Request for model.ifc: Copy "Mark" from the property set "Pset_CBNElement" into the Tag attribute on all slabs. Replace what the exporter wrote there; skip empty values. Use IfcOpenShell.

First a look at what the model holds.

```python
import ifcopenshell
import ifcopenshell.util.element

model = ifcopenshell.open("model.ifc")
print(model.schema)
slabs = model.by_type("IfcSlab")
print(len(slabs), "slabs")
for e in slabs[:8]:
    source = ifcopenshell.util.element.get_pset(e, "Pset_CBNElement", "Mark")
    target = e.Tag
    print(e.id(), repr(source), repr(target), sep=" | ")
```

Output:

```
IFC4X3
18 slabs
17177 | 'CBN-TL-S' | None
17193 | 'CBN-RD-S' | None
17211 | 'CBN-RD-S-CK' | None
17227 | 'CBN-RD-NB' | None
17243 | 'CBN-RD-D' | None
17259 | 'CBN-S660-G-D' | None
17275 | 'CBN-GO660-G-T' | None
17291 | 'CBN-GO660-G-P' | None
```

```python
import ifcopenshell
import ifcopenshell.util.element

model = ifcopenshell.open("model.ifc")

count = 0
for e in model.by_type("IfcSlab"):
    value = ifcopenshell.util.element.get_pset(e, "Pset_CBNElement", "Mark")
    current = e.Tag
    if not value or not value.strip() or current == value:
        continue
    e.Tag = value
    count += 1

print(count, "slabs updated")

model.write("model-out.ifc")
```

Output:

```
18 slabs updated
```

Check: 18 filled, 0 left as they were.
